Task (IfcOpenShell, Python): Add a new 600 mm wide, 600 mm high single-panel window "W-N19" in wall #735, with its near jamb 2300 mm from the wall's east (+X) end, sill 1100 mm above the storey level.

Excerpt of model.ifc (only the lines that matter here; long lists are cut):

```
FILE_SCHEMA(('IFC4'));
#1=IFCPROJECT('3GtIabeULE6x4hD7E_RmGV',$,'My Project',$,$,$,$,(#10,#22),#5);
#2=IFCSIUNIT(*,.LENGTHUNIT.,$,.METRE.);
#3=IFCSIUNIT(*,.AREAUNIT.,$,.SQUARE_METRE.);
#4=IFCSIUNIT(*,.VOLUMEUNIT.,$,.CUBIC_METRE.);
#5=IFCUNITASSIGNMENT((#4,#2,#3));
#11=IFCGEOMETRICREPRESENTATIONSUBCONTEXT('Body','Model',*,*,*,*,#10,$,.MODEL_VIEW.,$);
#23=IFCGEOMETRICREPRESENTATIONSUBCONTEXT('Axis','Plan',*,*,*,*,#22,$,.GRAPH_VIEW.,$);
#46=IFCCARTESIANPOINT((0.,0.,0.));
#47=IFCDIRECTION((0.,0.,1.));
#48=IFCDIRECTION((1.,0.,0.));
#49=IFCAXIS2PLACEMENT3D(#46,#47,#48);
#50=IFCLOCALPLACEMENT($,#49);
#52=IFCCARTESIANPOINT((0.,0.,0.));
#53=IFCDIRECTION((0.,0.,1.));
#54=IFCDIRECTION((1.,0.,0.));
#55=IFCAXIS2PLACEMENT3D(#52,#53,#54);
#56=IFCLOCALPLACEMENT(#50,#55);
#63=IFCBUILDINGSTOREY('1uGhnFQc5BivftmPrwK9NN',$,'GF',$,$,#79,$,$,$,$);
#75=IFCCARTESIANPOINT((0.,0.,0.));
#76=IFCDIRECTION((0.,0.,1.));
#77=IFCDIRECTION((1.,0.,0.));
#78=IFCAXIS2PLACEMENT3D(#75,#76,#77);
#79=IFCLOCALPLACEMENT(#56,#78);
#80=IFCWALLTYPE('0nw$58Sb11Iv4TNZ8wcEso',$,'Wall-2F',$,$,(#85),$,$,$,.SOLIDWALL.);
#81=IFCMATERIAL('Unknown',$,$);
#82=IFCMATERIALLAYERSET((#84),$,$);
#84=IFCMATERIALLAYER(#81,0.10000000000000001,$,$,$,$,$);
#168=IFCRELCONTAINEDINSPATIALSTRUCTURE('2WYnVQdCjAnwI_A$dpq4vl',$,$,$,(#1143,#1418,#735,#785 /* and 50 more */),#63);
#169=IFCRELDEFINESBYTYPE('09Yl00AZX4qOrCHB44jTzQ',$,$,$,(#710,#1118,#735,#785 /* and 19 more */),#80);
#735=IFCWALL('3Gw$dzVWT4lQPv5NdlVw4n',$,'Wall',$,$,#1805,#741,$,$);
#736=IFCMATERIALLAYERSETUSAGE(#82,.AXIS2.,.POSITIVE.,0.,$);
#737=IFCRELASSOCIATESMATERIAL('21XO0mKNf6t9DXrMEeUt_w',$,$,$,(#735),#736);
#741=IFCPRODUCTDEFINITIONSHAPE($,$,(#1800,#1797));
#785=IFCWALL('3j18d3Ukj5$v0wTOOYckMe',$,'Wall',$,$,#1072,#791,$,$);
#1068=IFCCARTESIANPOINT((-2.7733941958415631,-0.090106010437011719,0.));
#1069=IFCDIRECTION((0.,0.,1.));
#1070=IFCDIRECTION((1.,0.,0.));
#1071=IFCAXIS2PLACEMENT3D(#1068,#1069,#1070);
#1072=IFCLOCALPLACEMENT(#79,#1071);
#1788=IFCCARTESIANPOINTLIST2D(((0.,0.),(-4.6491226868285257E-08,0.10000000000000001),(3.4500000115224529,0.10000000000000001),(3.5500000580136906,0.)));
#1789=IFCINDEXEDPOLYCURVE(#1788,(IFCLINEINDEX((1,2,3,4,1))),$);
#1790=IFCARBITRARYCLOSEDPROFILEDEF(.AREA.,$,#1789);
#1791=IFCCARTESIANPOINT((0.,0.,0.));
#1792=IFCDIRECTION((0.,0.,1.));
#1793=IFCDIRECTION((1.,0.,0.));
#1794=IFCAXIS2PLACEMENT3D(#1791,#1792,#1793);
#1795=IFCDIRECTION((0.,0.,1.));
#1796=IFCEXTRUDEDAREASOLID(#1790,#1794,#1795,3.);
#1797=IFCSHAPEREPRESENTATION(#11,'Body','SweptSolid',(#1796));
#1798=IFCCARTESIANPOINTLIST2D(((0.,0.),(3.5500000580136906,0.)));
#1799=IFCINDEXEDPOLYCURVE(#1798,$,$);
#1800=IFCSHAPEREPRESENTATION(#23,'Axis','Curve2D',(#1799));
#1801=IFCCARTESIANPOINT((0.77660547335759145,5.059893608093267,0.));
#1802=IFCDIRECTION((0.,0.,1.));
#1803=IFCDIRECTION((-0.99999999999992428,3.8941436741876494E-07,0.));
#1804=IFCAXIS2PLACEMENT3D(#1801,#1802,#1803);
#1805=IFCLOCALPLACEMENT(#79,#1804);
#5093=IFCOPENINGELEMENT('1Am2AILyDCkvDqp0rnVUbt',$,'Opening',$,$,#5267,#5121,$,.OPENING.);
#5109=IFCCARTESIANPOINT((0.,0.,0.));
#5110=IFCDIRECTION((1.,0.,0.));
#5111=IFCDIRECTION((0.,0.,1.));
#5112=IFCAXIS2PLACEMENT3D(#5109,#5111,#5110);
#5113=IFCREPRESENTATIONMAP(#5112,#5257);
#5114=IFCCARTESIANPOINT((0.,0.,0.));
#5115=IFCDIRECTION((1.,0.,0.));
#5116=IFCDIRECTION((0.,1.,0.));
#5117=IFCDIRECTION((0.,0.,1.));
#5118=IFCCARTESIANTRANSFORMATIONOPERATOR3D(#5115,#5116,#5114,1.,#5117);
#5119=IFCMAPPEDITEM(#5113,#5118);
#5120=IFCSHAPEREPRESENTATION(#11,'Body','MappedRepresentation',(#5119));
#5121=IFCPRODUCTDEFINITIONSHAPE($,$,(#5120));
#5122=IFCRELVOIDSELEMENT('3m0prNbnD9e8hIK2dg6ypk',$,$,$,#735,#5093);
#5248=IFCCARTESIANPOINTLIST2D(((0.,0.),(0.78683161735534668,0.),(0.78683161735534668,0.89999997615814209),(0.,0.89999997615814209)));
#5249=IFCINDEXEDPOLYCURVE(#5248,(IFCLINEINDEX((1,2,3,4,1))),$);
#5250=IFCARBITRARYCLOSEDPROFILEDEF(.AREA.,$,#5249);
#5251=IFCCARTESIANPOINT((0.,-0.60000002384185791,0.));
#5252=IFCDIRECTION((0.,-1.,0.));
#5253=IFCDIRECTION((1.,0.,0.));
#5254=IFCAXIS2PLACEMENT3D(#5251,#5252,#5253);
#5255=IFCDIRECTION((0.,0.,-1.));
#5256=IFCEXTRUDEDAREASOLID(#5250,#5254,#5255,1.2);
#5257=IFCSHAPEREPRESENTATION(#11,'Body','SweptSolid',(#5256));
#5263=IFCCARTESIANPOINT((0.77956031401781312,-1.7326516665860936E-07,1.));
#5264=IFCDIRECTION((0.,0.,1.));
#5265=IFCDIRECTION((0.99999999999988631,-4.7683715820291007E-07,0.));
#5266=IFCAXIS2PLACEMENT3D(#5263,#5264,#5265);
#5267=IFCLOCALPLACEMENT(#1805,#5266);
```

```python
import numpy as np
import ifcopenshell
import ifcopenshell.api.feature
import ifcopenshell.api.geometry
import ifcopenshell.api.root
import ifcopenshell.api.spatial
import ifcopenshell.geom
import ifcopenshell.util.element
import ifcopenshell.util.placement
import ifcopenshell.util.representation
import ifcopenshell.util.shape
import ifcopenshell.util.unit

model = ifcopenshell.open("model.ifc")
unit_scale = ifcopenshell.util.unit.calculate_unit_scale(model)
settings = ifcopenshell.geom.settings()


def volume(element):
    """Net volume in cubic metres, openings subtracted."""
    shape = ifcopenshell.geom.create_shape(settings, element)
    return ifcopenshell.util.shape.get_volume(shape.geometry)


wall = model.by_guid("3Gw$dzVWT4lQPv5NdlVw4n")
storey = ifcopenshell.util.element.get_container(wall, ifc_class="IfcBuildingStorey")
context = ifcopenshell.util.representation.get_context(model, "Model", "Body", "MODEL_VIEW")
before = volume(wall)

width, height, from_end, sill = 0.6, 0.6, 2.3, 1.1  # metres

# The wall runs along its own X axis, and the end named is its -X end.
wall_shape = ifcopenshell.geom.create_shape(settings, wall)
x, y, z = ifcopenshell.util.shape.get_vertices(wall_shape.geometry).T
start = x.min() + from_end
face, thickness = float(y.min()), float(y.max() - y.min())
wall_matrix = ifcopenshell.util.placement.get_local_placement(wall.ObjectPlacement)
level = ifcopenshell.util.placement.get_local_placement(storey.ObjectPlacement)[2, 3]


def in_wall(x, y):
    """Placement at x, y metres in the wall's axes, at sill height."""
    matrix = wall_matrix.copy()
    matrix[:, 3] = wall_matrix @ np.array([x / unit_scale, y / unit_scale, 0.0, 1.0])
    matrix[2, 3] = level + sill / unit_scale
    return matrix


# Opening: a box that overshoots both wall faces by 50 mm.
opening = ifcopenshell.api.root.create_entity(model, ifc_class="IfcOpeningElement", predefined_type="OPENING")
box = ifcopenshell.api.geometry.add_wall_representation(
    model, context=context, length=width, height=height, thickness=thickness + 0.1
)
ifcopenshell.api.geometry.assign_representation(model, product=opening, representation=box)
ifcopenshell.api.geometry.edit_object_placement(model, product=opening, matrix=in_wall(start, face - 0.05), is_si=False)
ifcopenshell.api.feature.add_feature(model, feature=opening, element=wall)

window = ifcopenshell.api.root.create_entity(model, ifc_class="IfcWindow", name="W-N19", predefined_type="WINDOW")
window.OverallWidth, window.OverallHeight = width / unit_scale, height / unit_scale
window.PartitioningType = "SINGLE_PANEL"
body = ifcopenshell.api.geometry.add_window_representation(
    model,
    context=context,
    overall_width=window.OverallWidth,
    overall_height=window.OverallHeight,
    partition_type="SINGLE_PANEL",
)
ifcopenshell.api.geometry.assign_representation(model, product=window, representation=body)
ifcopenshell.api.spatial.assign_container(model, products=[window], relating_structure=storey)
ifcopenshell.api.feature.add_filling(model, opening=opening, element=window)

# Centre the window in the wall's thickness.
ifcopenshell.api.geometry.edit_object_placement(model, product=window, matrix=in_wall(start, face), is_si=False)
window_shape = ifcopenshell.geom.create_shape(settings, window)
depth = ifcopenshell.util.shape.get_vertices(window_shape.geometry)[:, 1]
offset = face + thickness / 2 - (depth.min() + depth.max()) / 2
ifcopenshell.api.geometry.edit_object_placement(model, product=window, matrix=in_wall(start, offset), is_si=False)

after = volume(wall)

print(f"wall volume {before:.3f} -> {after:.3f} m3")

model.write("model_edited.ifc")
```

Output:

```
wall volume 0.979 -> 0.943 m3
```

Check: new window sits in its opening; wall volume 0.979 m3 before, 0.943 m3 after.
